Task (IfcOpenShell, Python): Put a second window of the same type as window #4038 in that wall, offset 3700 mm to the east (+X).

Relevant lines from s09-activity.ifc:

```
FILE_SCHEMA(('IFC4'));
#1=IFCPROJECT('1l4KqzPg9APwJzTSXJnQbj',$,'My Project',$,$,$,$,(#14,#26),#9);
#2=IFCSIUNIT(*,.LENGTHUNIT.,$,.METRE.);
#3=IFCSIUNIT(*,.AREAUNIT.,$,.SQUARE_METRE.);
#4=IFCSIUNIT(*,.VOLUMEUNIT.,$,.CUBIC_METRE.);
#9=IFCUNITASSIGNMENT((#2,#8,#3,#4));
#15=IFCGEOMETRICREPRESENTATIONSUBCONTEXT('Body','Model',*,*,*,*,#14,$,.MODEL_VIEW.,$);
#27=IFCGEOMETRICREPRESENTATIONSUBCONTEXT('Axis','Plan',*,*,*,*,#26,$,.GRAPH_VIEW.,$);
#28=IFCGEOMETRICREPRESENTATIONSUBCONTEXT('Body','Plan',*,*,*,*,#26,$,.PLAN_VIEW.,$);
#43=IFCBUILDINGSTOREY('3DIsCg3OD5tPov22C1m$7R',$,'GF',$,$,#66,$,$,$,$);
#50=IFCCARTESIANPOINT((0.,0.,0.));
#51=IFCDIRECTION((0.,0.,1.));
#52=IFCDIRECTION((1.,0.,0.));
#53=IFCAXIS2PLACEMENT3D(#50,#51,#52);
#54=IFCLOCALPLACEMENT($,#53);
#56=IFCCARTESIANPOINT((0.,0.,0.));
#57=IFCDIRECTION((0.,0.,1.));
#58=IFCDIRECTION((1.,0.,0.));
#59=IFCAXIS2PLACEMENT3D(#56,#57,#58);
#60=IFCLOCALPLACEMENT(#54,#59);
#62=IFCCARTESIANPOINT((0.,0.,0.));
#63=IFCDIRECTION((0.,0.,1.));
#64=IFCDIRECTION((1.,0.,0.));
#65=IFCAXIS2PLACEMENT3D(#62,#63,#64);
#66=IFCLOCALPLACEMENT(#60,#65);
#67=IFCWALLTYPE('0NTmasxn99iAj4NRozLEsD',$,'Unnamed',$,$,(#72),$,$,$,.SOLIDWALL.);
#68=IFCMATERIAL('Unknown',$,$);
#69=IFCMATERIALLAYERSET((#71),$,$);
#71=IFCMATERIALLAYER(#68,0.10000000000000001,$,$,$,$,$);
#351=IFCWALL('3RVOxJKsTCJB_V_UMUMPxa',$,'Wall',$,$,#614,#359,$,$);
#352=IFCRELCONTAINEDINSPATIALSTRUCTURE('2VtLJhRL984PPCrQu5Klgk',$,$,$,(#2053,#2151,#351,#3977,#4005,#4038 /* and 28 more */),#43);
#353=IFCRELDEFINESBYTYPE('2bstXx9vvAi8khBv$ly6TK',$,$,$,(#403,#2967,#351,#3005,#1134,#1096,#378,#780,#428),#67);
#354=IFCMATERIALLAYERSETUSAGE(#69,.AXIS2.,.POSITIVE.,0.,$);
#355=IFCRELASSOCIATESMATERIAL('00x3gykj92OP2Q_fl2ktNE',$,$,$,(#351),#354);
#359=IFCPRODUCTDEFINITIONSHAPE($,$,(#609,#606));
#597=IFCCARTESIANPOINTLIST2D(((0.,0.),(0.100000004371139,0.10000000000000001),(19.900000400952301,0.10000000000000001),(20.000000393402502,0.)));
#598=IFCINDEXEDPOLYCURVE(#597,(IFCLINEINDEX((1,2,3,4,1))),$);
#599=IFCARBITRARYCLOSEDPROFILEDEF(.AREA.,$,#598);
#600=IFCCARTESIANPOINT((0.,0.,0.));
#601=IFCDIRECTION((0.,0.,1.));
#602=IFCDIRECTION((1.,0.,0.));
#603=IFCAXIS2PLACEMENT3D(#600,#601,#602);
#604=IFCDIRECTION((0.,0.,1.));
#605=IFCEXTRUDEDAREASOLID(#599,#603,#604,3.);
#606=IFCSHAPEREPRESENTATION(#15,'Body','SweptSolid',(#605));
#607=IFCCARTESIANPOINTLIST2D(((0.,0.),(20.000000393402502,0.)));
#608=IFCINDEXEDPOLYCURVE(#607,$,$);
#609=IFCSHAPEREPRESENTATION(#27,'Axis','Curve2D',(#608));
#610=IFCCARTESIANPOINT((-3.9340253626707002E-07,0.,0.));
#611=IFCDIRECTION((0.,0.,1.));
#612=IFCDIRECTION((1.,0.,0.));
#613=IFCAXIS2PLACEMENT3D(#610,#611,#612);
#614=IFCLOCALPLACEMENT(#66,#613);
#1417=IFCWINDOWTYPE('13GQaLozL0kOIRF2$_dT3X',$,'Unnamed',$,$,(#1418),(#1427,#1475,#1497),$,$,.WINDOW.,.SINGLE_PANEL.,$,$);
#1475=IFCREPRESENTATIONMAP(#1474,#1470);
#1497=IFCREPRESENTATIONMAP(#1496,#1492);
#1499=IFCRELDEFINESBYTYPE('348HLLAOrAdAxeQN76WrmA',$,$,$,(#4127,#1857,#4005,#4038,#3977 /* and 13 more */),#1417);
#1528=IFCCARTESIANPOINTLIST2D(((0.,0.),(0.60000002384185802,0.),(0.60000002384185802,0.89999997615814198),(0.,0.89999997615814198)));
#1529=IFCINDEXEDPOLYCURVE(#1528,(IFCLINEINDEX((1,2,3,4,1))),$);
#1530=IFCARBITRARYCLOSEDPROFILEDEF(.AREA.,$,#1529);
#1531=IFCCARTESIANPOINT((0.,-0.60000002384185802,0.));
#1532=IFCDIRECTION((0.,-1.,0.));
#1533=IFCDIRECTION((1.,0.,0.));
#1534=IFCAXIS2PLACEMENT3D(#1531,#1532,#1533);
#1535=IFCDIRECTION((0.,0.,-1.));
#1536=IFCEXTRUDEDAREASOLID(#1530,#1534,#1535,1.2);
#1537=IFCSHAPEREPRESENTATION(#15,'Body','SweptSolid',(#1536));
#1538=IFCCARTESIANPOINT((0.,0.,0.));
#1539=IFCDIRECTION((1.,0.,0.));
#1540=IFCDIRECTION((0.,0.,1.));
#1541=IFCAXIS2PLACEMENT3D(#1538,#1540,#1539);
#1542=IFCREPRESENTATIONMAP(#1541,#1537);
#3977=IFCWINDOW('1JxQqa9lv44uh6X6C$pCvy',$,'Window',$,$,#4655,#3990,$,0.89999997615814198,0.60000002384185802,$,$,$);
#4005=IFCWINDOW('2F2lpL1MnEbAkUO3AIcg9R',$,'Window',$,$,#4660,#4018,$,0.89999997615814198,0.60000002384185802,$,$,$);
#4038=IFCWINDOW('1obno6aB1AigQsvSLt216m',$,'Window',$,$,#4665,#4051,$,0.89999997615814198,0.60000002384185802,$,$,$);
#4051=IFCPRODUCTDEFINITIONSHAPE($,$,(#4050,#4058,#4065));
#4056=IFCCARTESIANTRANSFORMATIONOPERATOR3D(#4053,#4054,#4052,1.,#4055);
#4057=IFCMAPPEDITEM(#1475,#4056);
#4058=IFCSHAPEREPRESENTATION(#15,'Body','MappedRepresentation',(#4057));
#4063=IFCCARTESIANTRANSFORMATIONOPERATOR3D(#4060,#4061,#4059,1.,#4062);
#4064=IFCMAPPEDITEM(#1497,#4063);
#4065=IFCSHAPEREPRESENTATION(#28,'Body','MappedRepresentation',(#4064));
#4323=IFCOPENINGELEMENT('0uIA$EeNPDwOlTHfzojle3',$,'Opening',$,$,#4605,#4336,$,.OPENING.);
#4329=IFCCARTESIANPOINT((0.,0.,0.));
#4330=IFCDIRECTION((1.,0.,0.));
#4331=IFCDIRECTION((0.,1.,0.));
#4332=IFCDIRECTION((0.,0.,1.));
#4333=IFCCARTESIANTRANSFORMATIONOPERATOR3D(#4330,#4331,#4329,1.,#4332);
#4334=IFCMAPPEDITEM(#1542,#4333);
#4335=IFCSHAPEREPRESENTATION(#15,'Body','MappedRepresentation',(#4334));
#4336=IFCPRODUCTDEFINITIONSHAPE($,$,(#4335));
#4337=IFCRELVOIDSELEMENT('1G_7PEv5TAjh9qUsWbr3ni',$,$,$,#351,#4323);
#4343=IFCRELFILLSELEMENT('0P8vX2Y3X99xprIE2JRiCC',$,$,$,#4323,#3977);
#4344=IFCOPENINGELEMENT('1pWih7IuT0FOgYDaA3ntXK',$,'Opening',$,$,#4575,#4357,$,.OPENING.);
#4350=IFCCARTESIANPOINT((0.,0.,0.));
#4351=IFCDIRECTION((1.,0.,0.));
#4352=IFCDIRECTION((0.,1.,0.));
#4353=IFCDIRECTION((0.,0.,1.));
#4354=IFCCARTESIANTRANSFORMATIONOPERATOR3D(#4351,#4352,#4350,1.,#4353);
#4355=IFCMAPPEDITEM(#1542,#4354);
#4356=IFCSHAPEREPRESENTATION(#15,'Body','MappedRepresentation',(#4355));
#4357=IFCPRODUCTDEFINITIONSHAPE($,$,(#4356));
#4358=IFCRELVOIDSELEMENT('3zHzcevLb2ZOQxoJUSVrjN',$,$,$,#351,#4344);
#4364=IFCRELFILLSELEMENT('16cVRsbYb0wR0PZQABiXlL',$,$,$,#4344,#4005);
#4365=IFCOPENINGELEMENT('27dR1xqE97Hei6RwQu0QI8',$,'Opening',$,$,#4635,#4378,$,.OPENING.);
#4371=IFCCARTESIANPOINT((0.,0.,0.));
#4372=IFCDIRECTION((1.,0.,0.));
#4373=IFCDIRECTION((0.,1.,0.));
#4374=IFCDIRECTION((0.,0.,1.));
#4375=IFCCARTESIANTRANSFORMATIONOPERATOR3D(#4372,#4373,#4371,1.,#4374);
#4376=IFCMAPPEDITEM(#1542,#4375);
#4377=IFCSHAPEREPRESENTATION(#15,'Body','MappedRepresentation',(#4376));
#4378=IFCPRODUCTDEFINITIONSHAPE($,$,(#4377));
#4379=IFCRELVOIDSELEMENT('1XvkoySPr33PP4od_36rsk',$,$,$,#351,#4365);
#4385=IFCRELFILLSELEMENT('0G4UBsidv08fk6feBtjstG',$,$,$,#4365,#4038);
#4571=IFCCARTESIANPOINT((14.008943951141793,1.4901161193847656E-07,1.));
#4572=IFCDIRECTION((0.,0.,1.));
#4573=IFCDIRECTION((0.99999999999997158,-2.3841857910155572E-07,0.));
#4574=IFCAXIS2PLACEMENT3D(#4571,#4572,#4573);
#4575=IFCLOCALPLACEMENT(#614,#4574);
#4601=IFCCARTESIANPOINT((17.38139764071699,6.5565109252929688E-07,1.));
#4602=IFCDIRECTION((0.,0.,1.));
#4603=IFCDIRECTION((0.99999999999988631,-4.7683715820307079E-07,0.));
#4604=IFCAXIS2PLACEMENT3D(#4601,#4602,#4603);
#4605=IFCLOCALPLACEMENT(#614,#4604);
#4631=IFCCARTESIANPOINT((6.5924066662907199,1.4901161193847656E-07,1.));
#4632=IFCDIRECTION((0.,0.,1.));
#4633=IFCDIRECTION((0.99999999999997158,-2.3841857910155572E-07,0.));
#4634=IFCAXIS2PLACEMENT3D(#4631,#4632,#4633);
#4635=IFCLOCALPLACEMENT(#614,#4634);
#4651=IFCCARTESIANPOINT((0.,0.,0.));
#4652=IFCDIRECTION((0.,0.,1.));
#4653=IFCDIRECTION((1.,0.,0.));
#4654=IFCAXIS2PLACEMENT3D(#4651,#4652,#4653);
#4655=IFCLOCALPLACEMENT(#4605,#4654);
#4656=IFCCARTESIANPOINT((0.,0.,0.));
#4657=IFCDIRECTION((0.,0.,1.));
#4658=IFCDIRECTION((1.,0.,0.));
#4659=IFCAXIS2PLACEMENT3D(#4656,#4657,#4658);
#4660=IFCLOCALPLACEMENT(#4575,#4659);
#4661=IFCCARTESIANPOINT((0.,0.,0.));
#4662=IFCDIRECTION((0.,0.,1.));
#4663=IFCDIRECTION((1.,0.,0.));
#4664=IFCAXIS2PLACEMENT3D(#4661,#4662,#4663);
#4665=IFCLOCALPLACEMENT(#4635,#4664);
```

```python
import ifcopenshell
import ifcopenshell.api.feature
import ifcopenshell.api.geometry
import ifcopenshell.api.root
import ifcopenshell.geom
import ifcopenshell.util.element
import ifcopenshell.util.placement
import ifcopenshell.util.shape

model = ifcopenshell.open("s09-activity.ifc")
settings = ifcopenshell.geom.settings()


def volume(element):
    """Net volume in cubic metres, openings subtracted."""
    shape = ifcopenshell.geom.create_shape(settings, element)
    return ifcopenshell.util.shape.get_volume(shape.geometry)


window = model.by_guid("1obno6aB1AigQsvSLt216m")
opening = window.FillsVoids[0].RelatingOpeningElement
wall = opening.VoidsElements[0].RelatingBuildingElement
before = volume(wall)
shift = ifcopenshell.util.placement.get_local_placement(wall.ObjectPlacement)[:3, 0] * 3.7

# copy_class copies the void relationship, type, container and properties, but no geometry.
new_opening = ifcopenshell.api.root.copy_class(model, product=opening)
new_opening.Representation = ifcopenshell.util.element.copy_deep(
    model, opening.Representation, exclude=["IfcGeometricRepresentationContext", "IfcRepresentationMap"]
)
new_window = ifcopenshell.api.root.copy_class(model, product=window)
new_window.Representation = ifcopenshell.util.element.copy_deep(
    model, window.Representation, exclude=["IfcGeometricRepresentationContext", "IfcRepresentationMap"]
)
ifcopenshell.api.feature.add_filling(model, opening=new_opening, element=new_window)

for old, new in ((opening, new_opening), (window, new_window)):
    matrix = ifcopenshell.util.placement.get_local_placement(old.ObjectPlacement)
    matrix[:3, 3] += shift
    ifcopenshell.api.geometry.edit_object_placement(model, product=new, matrix=matrix, is_si=False)

after = volume(wall)

print(f"wall volume {before:.3f} -> {after:.3f} m3")

model.write("s09-activity-out.ifc")
```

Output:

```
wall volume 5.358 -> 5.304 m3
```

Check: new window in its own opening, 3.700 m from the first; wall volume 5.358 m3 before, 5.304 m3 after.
